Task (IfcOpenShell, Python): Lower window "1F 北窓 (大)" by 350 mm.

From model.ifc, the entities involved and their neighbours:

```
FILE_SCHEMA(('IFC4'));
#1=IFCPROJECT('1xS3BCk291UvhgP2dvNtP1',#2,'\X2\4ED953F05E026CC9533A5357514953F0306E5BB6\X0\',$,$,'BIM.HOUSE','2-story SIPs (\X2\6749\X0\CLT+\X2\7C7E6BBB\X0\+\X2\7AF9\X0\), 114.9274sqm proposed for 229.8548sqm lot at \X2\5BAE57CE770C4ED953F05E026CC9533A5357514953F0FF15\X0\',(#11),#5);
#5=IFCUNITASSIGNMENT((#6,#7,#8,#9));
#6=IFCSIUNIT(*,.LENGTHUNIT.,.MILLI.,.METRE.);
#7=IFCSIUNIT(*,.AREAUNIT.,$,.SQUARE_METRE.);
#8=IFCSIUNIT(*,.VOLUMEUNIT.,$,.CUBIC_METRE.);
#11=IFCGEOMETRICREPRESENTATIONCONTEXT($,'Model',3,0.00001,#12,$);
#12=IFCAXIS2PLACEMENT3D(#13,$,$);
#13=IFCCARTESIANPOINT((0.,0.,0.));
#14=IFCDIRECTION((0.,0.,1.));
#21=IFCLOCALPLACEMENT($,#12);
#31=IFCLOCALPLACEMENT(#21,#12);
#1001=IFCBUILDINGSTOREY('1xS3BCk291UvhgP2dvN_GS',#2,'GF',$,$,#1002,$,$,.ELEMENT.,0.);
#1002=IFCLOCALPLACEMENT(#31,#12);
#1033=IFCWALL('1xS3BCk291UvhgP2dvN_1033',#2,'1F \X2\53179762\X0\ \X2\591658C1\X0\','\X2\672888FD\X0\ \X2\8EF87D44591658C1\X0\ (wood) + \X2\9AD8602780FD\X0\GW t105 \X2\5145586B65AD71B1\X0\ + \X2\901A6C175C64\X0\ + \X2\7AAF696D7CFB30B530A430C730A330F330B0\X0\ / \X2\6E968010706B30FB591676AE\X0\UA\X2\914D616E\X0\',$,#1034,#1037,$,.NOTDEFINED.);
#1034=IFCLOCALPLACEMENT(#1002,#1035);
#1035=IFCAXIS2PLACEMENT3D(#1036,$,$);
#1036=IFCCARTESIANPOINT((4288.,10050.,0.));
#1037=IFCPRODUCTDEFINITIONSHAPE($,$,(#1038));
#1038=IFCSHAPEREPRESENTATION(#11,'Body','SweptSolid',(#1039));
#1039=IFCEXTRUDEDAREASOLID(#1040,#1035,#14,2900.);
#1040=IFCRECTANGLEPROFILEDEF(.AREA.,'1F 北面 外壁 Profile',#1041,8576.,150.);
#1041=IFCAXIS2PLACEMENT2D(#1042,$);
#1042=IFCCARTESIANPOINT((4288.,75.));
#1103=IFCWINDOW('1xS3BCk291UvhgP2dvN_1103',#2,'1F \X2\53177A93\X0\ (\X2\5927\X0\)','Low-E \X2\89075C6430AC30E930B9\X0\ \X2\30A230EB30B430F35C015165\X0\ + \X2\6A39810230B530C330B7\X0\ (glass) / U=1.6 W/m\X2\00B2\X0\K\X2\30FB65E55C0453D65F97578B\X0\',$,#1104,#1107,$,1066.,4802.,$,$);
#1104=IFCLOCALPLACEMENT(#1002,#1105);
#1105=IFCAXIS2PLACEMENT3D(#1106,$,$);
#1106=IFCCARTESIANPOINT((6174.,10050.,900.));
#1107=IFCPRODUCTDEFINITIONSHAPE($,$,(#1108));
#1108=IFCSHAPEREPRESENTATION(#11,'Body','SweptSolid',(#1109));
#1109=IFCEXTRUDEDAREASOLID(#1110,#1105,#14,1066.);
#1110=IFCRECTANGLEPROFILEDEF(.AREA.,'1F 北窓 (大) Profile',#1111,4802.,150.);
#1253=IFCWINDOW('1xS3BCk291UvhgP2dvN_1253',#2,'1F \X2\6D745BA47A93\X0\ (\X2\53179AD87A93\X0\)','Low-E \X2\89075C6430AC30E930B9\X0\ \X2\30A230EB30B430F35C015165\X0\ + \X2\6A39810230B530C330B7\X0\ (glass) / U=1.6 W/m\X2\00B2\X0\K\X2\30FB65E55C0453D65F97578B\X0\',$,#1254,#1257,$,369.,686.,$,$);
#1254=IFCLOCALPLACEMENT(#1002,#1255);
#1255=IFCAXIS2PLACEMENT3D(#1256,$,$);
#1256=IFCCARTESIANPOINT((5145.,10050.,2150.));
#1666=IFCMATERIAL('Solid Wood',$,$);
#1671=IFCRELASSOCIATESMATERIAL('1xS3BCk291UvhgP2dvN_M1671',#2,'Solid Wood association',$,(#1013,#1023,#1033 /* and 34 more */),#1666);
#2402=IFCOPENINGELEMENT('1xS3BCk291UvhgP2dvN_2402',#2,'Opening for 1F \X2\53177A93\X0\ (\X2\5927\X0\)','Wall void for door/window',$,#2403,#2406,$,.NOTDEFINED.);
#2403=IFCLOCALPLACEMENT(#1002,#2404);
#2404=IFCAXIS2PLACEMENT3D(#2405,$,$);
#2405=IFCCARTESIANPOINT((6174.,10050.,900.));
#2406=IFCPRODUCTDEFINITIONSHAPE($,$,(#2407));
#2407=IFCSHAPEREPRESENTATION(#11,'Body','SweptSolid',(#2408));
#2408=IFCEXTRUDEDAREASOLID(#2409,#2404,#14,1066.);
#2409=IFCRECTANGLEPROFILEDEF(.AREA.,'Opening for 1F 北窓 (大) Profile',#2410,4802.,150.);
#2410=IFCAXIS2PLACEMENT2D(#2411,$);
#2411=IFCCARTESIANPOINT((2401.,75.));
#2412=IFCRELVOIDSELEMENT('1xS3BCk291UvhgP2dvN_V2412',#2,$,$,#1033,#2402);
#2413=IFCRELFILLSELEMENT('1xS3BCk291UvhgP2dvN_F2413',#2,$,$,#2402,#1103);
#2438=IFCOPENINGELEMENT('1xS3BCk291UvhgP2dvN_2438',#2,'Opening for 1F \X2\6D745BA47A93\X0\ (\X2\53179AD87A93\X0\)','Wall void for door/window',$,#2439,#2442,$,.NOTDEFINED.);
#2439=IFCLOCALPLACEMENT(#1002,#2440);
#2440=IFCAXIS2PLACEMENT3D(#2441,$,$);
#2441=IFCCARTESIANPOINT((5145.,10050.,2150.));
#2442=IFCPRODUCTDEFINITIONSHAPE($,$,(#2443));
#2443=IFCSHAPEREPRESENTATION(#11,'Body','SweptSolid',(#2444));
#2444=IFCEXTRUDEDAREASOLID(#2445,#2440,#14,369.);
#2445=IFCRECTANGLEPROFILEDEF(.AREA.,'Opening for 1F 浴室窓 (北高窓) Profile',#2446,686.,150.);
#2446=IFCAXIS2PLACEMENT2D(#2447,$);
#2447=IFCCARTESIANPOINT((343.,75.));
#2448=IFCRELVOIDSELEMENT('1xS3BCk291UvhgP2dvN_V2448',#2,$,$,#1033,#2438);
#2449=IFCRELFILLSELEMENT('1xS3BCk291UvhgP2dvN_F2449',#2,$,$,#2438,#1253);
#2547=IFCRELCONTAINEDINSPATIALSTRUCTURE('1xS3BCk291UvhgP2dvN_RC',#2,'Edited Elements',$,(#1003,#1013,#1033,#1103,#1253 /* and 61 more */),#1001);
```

```python
import numpy as np
import ifcopenshell
import ifcopenshell.api.geometry
import ifcopenshell.util.placement
import ifcopenshell.util.unit

model = ifcopenshell.open("model.ifc")
unit_scale = ifcopenshell.util.unit.calculate_unit_scale(model)

window = model.by_guid("1xS3BCk291UvhgP2dvN_1103")
opening = window.FillsVoids[0].RelatingOpeningElement
dz = -0.35 / unit_scale

shift = np.array([0.0, 0.0, dz])
# The window is not placed relative to its opening, so move both.
for product in (opening, window):
    matrix = ifcopenshell.util.placement.get_local_placement(product.ObjectPlacement)
    matrix[:3, 3] += shift
    ifcopenshell.api.geometry.edit_object_placement(model, product=product, matrix=matrix, is_si=False)

print(f"moved by {dz * unit_scale:+.3f} m")

model.write("model_rev.ifc")
```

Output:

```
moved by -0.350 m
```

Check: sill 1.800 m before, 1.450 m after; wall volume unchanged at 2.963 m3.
